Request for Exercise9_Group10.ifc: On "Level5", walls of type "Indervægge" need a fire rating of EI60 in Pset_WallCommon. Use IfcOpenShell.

First a look at what the model holds.

```python
import ifcopenshell
import ifcopenshell.util.element

model = ifcopenshell.open("Exercise9_Group10.ifc")
print(model.schema)
storey = next(s for s in model.by_type("IfcBuildingStorey") if s.Name == "Level5")
walls = [e for e in ifcopenshell.util.element.get_decomposition(storey) if e.is_a("IfcWall")]
seen = {}
for e in walls:
    element_type = ifcopenshell.util.element.get_type(e)
    key = (element_type.Name if element_type != e and element_type else None, ifcopenshell.util.element.get_pset(e, "Pset_WallCommon", "FireRating"))
    seen[key] = seen.get(key, 0) + 1
for (name, value), count in sorted(seen.items(), key=str):
    print(count, "x", name, "|", value)
```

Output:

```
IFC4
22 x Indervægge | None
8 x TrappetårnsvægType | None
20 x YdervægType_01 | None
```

```python
import ifcopenshell
import ifcopenshell.api.pset
import ifcopenshell.util.element

model = ifcopenshell.open("Exercise9_Group10.ifc")

storey = next(s for s in model.by_type("IfcBuildingStorey") if s.Name == "Level5")
walls = [e for e in ifcopenshell.util.element.get_decomposition(storey) if e.is_a("IfcWall")]

count = 0
for e in walls:
    element_type = ifcopenshell.util.element.get_type(e)
    if element_type in (None, e) or element_type.Name != "Indervægge":
        continue
    # add_pset returns the element's existing set when there is one.
    pset = ifcopenshell.api.pset.add_pset(model, product=e, name="Pset_WallCommon")
    ifcopenshell.api.pset.edit_pset(model, pset=pset, properties={"FireRating": "EI60"})
    count += 1

print(count, "walls updated")

model.write("Exercise9_Group10-out.ifc")
```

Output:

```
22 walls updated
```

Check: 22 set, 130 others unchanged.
